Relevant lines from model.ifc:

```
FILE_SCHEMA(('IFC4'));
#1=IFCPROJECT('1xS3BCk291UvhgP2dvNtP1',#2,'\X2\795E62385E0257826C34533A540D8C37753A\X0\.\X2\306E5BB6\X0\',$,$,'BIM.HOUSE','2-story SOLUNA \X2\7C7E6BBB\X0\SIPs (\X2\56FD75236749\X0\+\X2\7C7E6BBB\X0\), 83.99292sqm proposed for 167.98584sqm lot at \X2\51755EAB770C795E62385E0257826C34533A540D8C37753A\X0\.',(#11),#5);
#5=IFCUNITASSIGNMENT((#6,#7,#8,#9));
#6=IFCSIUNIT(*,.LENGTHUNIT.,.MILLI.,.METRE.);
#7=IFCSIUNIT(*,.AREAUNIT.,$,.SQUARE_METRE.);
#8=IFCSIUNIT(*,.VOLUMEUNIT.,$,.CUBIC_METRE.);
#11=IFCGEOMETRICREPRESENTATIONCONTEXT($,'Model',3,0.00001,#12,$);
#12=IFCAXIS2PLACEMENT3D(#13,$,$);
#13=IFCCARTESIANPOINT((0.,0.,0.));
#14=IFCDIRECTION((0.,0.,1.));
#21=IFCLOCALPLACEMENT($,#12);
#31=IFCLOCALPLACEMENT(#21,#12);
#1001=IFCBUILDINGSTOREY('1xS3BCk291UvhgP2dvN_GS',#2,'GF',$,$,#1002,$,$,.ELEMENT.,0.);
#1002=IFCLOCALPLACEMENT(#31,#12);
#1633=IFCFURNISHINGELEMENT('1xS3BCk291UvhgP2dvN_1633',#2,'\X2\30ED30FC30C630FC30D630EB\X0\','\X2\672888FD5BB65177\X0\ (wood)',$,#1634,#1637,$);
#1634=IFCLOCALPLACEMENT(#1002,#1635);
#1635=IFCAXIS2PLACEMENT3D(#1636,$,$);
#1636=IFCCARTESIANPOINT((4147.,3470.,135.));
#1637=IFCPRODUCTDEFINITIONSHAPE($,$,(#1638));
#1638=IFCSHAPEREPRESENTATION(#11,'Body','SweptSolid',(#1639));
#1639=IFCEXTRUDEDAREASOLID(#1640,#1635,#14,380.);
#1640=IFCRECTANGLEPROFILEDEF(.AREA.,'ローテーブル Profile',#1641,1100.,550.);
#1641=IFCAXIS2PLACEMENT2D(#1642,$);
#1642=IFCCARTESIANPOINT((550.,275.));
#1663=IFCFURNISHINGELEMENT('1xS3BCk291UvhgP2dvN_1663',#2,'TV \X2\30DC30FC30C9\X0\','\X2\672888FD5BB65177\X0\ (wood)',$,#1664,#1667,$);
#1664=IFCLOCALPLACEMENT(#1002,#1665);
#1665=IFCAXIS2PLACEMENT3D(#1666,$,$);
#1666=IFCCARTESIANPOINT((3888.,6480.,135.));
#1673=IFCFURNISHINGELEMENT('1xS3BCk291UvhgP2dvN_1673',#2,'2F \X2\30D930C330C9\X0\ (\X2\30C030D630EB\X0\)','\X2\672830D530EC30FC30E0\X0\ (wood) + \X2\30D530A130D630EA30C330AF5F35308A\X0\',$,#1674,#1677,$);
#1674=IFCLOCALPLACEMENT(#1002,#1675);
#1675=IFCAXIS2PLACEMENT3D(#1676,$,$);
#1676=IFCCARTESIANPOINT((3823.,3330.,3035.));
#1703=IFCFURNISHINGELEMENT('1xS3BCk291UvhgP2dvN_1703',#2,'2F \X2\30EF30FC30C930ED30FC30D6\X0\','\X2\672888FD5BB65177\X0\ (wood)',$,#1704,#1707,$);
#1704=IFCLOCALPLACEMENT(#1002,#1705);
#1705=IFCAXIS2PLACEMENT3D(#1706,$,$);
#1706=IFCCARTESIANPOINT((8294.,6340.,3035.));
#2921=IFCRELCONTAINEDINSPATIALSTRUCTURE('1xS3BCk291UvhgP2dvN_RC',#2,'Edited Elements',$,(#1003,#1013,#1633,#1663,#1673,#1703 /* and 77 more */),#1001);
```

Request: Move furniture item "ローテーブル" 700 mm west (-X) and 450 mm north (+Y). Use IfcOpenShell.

```python
import ifcopenshell
import ifcopenshell.api.geometry
import ifcopenshell.util.placement
import ifcopenshell.util.unit

model = ifcopenshell.open("model.ifc")
unit_scale = ifcopenshell.util.unit.calculate_unit_scale(model)

item = model.by_guid("1xS3BCk291UvhgP2dvN_1633")
matrix = ifcopenshell.util.placement.get_local_placement(item.ObjectPlacement)
matrix[0, 3] -= 0.7 / unit_scale
matrix[1, 3] += 0.45 / unit_scale
ifcopenshell.api.geometry.edit_object_placement(model, product=item, matrix=matrix, is_si=False)

print(ifcopenshell.util.placement.get_local_placement(item.ObjectPlacement).round(3) + 0.0)

model.write("model_v2.ifc")
```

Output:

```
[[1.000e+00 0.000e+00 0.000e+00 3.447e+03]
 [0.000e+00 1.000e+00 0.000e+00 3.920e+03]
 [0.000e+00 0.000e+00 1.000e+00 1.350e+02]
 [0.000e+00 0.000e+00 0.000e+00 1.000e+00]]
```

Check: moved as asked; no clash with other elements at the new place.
